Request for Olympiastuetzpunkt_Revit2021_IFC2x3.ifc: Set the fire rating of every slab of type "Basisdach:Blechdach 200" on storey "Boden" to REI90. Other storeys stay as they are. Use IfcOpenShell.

First a look at what the model holds.

```python
import ifcopenshell
import ifcopenshell.util.element

model = ifcopenshell.open("Olympiastuetzpunkt_Revit2021_IFC2x3.ifc")
print(model.schema)
storey = next(s for s in model.by_type("IfcBuildingStorey") if s.Name == "Boden")
slabs = [e for e in ifcopenshell.util.element.get_decomposition(storey) if e.is_a("IfcSlab")]
seen = {}
for e in slabs:
    element_type = ifcopenshell.util.element.get_type(e)
    key = (element_type.Name if element_type != e and element_type else None, ifcopenshell.util.element.get_pset(e, "Pset_SlabCommon", "FireRating"))
    seen[key] = seen.get(key, 0) + 1
for (name, value), count in sorted(seen.items(), key=str):
    print(count, "x", name, "|", value)
```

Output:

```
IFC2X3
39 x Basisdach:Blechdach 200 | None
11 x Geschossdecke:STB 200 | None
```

```python
import ifcopenshell
import ifcopenshell.api.pset
import ifcopenshell.util.element

model = ifcopenshell.open("Olympiastuetzpunkt_Revit2021_IFC2x3.ifc")

storey = next(s for s in model.by_type("IfcBuildingStorey") if s.Name == "Boden")
slabs = [e for e in ifcopenshell.util.element.get_decomposition(storey) if e.is_a("IfcSlab")]

count = 0
for e in slabs:
    element_type = ifcopenshell.util.element.get_type(e)
    if element_type in (None, e) or element_type.Name != "Basisdach:Blechdach 200":
        continue
    # add_pset returns the element's existing set when there is one.
    pset = ifcopenshell.api.pset.add_pset(model, product=e, name="Pset_SlabCommon")
    ifcopenshell.api.pset.edit_pset(model, pset=pset, properties={"FireRating": "REI90"})
    count += 1

print(count, "slabs updated")

model.write("Olympiastuetzpunkt_Revit2021_IFC2x3_updated.ifc")
```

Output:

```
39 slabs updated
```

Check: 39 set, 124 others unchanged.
